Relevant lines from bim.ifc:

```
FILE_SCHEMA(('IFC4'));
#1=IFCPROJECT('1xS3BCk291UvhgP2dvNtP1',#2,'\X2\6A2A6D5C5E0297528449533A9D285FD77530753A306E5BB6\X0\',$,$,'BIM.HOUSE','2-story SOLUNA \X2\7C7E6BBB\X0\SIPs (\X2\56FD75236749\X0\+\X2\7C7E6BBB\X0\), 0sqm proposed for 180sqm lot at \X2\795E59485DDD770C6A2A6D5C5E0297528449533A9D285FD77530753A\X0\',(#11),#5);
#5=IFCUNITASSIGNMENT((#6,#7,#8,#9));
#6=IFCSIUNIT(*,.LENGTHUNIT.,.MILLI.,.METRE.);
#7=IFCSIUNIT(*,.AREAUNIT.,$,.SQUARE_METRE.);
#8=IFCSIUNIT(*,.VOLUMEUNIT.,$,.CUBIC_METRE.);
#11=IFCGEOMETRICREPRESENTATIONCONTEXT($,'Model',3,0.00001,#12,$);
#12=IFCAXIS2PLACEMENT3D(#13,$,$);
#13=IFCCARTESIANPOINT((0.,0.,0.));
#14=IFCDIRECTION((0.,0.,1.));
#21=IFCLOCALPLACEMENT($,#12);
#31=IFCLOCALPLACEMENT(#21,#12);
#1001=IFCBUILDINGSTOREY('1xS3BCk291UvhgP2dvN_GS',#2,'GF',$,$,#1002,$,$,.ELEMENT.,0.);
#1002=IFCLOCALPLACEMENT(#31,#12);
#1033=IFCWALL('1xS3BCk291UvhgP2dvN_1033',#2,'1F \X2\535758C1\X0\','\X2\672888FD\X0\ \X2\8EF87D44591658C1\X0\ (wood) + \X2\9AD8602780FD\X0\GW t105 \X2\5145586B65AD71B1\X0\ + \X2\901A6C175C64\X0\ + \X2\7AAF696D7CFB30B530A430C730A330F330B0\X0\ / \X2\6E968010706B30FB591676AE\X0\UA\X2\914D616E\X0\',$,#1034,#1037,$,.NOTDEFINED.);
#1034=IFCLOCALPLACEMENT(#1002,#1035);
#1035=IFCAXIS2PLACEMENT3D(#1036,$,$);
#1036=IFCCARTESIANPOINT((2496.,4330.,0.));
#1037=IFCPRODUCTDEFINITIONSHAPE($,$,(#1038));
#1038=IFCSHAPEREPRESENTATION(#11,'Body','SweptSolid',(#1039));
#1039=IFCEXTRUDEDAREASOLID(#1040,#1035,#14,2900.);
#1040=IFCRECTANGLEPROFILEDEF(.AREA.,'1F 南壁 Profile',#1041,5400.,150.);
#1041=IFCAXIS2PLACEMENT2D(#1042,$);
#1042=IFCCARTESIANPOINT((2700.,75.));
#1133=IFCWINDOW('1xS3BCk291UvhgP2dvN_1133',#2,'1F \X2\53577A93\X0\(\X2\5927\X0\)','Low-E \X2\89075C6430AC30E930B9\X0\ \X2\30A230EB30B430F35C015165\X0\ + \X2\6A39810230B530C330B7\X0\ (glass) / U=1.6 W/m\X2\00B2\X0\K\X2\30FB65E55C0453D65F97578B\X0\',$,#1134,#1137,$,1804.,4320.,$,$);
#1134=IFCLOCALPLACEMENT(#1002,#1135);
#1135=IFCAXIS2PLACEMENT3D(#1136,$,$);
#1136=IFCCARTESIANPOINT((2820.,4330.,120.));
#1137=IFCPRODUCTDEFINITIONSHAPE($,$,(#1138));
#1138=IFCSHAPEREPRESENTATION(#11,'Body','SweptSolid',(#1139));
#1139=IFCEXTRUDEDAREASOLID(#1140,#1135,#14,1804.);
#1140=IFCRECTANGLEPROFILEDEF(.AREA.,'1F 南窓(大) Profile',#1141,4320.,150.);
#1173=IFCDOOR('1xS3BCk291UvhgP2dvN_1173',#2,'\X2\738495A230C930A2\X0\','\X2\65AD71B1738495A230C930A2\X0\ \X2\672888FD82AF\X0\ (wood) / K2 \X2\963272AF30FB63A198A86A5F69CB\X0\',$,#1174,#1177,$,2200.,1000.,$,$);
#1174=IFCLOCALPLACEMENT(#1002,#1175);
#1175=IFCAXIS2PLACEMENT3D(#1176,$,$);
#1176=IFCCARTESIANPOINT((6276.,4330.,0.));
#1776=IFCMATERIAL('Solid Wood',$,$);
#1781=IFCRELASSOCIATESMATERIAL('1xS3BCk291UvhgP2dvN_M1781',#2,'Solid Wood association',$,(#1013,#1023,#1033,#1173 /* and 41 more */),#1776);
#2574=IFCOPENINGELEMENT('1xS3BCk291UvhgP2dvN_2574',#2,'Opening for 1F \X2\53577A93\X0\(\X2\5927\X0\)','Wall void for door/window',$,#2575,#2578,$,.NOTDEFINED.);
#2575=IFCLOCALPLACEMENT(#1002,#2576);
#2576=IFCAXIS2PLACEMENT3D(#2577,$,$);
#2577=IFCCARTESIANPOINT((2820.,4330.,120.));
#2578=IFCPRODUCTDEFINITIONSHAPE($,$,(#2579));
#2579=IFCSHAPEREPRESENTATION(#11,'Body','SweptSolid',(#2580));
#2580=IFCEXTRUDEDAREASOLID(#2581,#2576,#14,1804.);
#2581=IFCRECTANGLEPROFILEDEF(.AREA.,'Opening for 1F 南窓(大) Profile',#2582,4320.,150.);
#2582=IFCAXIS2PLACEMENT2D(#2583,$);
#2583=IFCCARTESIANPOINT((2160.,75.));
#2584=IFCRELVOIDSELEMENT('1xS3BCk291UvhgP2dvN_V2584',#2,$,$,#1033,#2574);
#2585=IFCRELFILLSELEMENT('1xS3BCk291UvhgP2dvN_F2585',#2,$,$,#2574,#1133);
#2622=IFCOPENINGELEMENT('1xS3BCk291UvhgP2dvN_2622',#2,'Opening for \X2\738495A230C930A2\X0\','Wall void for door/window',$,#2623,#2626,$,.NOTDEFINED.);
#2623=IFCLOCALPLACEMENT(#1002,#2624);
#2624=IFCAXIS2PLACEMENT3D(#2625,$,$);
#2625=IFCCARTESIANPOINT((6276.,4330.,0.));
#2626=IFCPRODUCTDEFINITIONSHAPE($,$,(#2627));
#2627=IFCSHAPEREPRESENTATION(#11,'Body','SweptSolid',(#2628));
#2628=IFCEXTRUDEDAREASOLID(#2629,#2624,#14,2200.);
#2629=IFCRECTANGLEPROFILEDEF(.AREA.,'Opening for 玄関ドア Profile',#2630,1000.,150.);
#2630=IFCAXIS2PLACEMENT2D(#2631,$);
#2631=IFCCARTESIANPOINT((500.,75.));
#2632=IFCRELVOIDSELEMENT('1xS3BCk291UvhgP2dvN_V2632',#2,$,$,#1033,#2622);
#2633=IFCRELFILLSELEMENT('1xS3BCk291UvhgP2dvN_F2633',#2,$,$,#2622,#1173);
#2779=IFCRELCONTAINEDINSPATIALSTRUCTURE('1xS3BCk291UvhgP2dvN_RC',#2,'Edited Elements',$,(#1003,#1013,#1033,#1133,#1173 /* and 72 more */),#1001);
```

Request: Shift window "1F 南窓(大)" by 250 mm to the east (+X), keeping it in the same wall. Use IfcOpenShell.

```python
import ifcopenshell
import ifcopenshell.api.geometry
import ifcopenshell.util.placement

model = ifcopenshell.open("bim.ifc")

window = model.by_guid("1xS3BCk291UvhgP2dvN_1133")
opening = window.FillsVoids[0].RelatingOpeningElement
wall = opening.VoidsElements[0].RelatingBuildingElement

wall_matrix = ifcopenshell.util.placement.get_local_placement(wall.ObjectPlacement)
shift = wall_matrix[:3, 0] * 250.0
before = ifcopenshell.util.placement.get_local_placement(window.ObjectPlacement)[:3, 3].copy()

# The window is not placed relative to its opening, so move both.
for product in (opening, window):
    matrix = ifcopenshell.util.placement.get_local_placement(product.ObjectPlacement)
    matrix[:3, 3] += shift
    ifcopenshell.api.geometry.edit_object_placement(model, product=product, matrix=matrix, is_si=False)

after = ifcopenshell.util.placement.get_local_placement(window.ObjectPlacement)[:3, 3]
print("window moved by", (after - before).round(3) + 0.0)

model.write("bim_edited.ifc")
```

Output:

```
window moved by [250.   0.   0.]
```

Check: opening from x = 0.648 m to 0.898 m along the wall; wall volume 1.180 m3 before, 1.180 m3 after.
